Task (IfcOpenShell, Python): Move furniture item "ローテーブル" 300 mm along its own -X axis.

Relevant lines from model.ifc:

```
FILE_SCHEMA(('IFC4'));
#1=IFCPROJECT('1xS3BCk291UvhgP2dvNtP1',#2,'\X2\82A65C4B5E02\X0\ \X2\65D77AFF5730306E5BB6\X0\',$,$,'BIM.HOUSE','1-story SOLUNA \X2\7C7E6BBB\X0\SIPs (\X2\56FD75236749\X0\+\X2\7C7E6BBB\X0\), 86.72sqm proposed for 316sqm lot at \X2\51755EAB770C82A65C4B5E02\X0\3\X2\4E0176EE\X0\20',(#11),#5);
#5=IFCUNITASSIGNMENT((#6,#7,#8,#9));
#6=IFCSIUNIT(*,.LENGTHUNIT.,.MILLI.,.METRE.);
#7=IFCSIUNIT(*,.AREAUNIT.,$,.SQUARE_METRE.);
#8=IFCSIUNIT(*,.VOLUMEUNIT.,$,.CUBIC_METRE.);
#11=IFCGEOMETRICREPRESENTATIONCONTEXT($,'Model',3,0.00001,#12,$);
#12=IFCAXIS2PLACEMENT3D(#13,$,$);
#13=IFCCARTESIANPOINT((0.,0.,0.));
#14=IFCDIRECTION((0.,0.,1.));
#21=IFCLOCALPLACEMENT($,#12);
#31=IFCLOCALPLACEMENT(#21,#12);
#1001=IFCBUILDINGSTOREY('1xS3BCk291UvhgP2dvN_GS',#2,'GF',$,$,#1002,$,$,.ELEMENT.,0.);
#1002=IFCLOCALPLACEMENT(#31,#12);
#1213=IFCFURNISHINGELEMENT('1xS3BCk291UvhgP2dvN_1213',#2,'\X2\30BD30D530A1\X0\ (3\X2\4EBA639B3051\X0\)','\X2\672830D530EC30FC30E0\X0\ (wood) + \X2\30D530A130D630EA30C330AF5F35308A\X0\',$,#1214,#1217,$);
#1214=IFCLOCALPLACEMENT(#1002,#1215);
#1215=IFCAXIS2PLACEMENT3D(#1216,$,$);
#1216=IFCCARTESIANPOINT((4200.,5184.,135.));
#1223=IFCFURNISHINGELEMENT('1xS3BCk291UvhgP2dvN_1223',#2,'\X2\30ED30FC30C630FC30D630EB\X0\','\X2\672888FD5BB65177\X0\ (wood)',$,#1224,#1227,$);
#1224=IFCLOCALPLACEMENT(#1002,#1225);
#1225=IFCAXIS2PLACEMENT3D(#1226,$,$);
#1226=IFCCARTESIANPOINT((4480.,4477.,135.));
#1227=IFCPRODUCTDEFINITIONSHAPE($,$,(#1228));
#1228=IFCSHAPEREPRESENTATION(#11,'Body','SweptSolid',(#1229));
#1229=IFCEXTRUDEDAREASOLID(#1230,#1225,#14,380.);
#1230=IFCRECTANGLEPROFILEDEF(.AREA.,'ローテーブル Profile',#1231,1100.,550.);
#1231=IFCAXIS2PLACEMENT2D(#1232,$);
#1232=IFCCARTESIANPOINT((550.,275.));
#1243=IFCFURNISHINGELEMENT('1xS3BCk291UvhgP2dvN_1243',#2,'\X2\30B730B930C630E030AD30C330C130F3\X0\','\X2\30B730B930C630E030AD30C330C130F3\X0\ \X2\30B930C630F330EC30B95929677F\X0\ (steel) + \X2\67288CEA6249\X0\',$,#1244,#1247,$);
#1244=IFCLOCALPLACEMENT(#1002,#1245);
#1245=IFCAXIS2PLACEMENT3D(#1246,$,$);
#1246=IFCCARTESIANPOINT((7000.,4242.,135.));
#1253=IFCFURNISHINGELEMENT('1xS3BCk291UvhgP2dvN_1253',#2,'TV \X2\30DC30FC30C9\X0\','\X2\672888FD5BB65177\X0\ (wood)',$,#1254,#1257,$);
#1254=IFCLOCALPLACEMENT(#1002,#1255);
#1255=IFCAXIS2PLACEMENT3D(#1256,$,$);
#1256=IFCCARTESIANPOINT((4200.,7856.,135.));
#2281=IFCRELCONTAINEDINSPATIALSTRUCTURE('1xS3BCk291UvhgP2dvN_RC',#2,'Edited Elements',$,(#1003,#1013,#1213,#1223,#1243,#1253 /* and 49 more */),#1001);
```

```python
import ifcopenshell
import ifcopenshell.api.geometry
import ifcopenshell.util.placement
import ifcopenshell.util.unit

model = ifcopenshell.open("model.ifc")
unit_scale = ifcopenshell.util.unit.calculate_unit_scale(model)

item = model.by_guid("1xS3BCk291UvhgP2dvN_1223")
matrix = ifcopenshell.util.placement.get_local_placement(item.ObjectPlacement)
matrix[:3, 3] -= matrix[:3, 0] * 0.3 / unit_scale
ifcopenshell.api.geometry.edit_object_placement(model, product=item, matrix=matrix, is_si=False)

print(ifcopenshell.util.placement.get_local_placement(item.ObjectPlacement).round(3) + 0.0)

model.write("model_updated.ifc")
```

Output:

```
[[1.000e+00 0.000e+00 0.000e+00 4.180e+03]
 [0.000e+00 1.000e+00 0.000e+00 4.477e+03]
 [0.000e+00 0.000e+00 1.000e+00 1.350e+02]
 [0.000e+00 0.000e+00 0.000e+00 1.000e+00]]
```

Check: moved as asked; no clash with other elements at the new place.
